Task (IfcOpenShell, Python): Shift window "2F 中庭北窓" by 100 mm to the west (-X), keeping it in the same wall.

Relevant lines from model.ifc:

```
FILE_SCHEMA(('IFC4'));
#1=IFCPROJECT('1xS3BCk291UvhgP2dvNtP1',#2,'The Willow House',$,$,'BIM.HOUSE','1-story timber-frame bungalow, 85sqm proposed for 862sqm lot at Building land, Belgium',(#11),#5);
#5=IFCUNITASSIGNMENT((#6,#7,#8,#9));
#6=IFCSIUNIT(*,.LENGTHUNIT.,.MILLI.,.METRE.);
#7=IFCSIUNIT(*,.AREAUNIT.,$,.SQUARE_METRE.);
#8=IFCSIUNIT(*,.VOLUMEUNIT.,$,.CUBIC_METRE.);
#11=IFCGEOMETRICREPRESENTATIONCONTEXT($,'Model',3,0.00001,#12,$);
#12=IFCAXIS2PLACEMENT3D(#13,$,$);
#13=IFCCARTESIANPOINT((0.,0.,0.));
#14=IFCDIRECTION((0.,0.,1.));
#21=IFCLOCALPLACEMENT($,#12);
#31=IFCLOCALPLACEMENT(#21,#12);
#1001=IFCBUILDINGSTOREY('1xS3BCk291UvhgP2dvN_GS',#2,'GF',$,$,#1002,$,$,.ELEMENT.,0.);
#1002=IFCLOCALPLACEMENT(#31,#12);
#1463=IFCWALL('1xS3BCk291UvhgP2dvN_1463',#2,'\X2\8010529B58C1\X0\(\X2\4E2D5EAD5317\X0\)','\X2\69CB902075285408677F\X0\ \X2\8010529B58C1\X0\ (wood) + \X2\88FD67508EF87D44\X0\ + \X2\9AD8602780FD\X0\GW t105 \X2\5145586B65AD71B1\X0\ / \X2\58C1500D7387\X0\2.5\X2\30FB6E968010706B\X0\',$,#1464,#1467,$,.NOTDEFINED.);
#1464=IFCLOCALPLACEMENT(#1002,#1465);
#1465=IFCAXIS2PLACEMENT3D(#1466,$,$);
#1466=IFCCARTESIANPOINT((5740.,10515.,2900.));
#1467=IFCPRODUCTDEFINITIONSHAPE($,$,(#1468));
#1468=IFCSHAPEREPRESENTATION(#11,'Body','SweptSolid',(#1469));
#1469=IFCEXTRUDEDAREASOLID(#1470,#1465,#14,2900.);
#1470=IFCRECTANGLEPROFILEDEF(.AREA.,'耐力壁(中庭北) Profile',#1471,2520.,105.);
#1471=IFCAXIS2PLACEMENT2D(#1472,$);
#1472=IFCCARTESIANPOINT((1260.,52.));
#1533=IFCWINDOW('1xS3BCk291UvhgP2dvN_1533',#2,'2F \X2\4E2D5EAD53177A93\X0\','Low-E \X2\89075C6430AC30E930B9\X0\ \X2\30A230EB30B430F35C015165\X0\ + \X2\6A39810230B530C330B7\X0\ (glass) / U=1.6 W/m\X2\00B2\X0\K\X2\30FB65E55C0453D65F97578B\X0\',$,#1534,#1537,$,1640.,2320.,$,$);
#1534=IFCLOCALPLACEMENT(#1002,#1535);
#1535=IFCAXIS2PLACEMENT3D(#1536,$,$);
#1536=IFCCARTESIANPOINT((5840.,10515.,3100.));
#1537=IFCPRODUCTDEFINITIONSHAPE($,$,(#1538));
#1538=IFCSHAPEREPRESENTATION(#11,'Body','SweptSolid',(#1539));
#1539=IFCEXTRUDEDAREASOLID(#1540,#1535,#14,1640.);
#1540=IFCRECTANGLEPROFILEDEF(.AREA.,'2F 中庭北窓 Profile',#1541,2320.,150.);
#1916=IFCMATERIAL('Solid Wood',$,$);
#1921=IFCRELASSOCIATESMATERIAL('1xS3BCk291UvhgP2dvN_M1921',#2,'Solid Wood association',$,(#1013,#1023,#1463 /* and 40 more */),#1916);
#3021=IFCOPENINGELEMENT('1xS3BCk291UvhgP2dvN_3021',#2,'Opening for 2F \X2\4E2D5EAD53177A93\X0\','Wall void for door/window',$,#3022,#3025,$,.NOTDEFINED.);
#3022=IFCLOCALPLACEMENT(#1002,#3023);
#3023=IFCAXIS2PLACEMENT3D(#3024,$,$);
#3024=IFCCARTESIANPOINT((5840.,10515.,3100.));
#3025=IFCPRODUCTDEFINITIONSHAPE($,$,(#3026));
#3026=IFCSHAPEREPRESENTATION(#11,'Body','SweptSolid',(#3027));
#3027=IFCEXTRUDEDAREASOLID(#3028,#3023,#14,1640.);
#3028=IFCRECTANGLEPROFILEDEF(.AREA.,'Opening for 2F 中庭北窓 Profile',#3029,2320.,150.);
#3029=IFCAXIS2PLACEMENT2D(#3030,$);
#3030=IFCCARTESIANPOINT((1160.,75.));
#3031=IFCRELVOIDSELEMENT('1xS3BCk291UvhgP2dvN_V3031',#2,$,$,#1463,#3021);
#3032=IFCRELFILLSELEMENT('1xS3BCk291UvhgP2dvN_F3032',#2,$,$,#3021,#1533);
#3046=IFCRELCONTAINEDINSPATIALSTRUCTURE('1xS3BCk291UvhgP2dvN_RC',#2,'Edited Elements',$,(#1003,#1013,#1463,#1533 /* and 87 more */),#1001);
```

```python
import ifcopenshell
import ifcopenshell.api.geometry
import ifcopenshell.util.placement
import ifcopenshell.util.unit

model = ifcopenshell.open("model.ifc")
unit_scale = ifcopenshell.util.unit.calculate_unit_scale(model)

window = model.by_id(1533)
opening = window.FillsVoids[0].RelatingOpeningElement
wall = opening.VoidsElements[0].RelatingBuildingElement

wall_matrix = ifcopenshell.util.placement.get_local_placement(wall.ObjectPlacement)
shift = wall_matrix[:3, 0] * -0.1 / unit_scale
before = ifcopenshell.util.placement.get_local_placement(window.ObjectPlacement)[:3, 3].copy()

# The window is not placed relative to its opening, so move both.
for product in (opening, window):
    matrix = ifcopenshell.util.placement.get_local_placement(product.ObjectPlacement)
    matrix[:3, 3] += shift
    ifcopenshell.api.geometry.edit_object_placement(model, product=product, matrix=matrix, is_si=False)

after = ifcopenshell.util.placement.get_local_placement(window.ObjectPlacement)[:3, 3]
print("window moved by", (after - before).round(3) + 0.0)

model.write("model_updated.ifc")
```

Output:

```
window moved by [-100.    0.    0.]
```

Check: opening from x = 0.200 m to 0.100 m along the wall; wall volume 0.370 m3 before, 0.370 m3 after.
